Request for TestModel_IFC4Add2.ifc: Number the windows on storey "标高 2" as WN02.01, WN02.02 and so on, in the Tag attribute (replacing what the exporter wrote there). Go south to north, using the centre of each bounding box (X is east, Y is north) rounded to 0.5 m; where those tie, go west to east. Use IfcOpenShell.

First a look at what the model holds.

```python
import ifcopenshell
import ifcopenshell.util.element
import ifcopenshell.util.placement

model = ifcopenshell.open("TestModel_IFC4Add2.ifc")
print(model.schema)
storey = next(s for s in model.by_type("IfcBuildingStorey") if s.Name == "标高 2")
windows = [e for e in ifcopenshell.util.element.get_decomposition(storey) if e.is_a("IfcWindow")]
for e in sorted(windows, key=lambda e: e.id()):
    origin = ifcopenshell.util.placement.get_local_placement(e.ObjectPlacement)[:3, 3]
    print(e.id(), e.Tag, e.Name, origin.round(2) + 0.0, sep=" | ")
```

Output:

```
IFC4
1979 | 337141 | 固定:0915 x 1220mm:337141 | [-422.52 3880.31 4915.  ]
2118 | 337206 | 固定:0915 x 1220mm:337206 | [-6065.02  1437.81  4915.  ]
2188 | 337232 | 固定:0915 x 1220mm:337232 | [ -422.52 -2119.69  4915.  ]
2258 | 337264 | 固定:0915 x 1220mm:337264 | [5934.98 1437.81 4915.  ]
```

```python
import ifcopenshell
import ifcopenshell.geom
import ifcopenshell.util.element
import ifcopenshell.util.shape

model = ifcopenshell.open("TestModel_IFC4Add2.ifc")
settings = ifcopenshell.geom.settings()
settings.set("use-world-coords", True)


def centre(element):
    shape = ifcopenshell.geom.create_shape(settings, element)
    return ifcopenshell.util.shape.get_bbox_centroid(shape.geometry)


storey = next(s for s in model.by_type("IfcBuildingStorey") if s.Name == "标高 2")
windows = [e for e in ifcopenshell.util.element.get_decomposition(storey) if e.is_a("IfcWindow")]

# Insertion points can sit at a corner or the storey origin, so sort by the geometry (in metres).
centres = {e: centre(e) for e in windows}
windows.sort(key=lambda e: (round(centres[e][1] / 0.5), centres[e][0]))

for i, e in enumerate(windows, start=1):
    number = f"WN02.{i:02d}"
    e.Tag = number
    print(e.id(), number)

model.write("TestModel_IFC4Add2_rev.ifc")
```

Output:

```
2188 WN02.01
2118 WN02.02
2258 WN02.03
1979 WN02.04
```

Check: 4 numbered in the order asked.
